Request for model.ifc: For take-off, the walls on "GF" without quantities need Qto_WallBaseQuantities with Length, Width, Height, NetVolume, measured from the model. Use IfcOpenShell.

First a look at what the model holds.

```python
import ifcopenshell
import ifcopenshell.util.element
import ifcopenshell.util.unit

model = ifcopenshell.open("model.ifc")
print(model.schema)
for unit_type in ("LENGTHUNIT", "AREAUNIT", "VOLUMEUNIT"):
    print(unit_type, ifcopenshell.util.unit.calculate_unit_scale(model, unit_type))
storey = next(s for s in model.by_type("IfcBuildingStorey") if s.Name == "GF")
walls = [e for e in ifcopenshell.util.element.get_decomposition(storey) if e.is_a("IfcWall")]
for e in sorted(walls, key=lambda e: e.id()):
    print(e.id(), e.is_a(), e.Name, list(ifcopenshell.util.element.get_psets(e, qtos_only=True)), sep=" | ")
```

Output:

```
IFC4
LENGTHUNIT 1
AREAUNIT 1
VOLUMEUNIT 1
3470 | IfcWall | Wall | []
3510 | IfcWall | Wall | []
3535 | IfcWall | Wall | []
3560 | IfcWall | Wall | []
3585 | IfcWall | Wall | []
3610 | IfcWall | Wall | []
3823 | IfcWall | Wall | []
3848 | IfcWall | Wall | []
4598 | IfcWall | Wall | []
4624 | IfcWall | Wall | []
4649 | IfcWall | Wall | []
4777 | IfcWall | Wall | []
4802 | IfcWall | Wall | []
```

```python
import ifcopenshell
import ifcopenshell.api.pset
import ifcopenshell.geom
import ifcopenshell.util.element
import ifcopenshell.util.shape
import ifcopenshell.util.unit

model = ifcopenshell.open("model.ifc")
unit_scale = ifcopenshell.util.unit.calculate_unit_scale(model)
volume_scale = ifcopenshell.util.unit.calculate_unit_scale(model, "VOLUMEUNIT")
settings = ifcopenshell.geom.settings()

storey = next(s for s in model.by_type("IfcBuildingStorey") if s.Name == "GF")
walls = [e for e in ifcopenshell.util.element.get_decomposition(storey) if e.is_a("IfcWall")]

for e in sorted(walls, key=lambda e: e.id()):
    if ifcopenshell.util.element.get_psets(e, qtos_only=True, should_inherit=False):
        continue
    # Geometry comes back in metres, in the element's own axes.
    shape = ifcopenshell.geom.create_shape(settings, e)
    values = {
        "Length": ifcopenshell.util.shape.get_x(shape.geometry) / unit_scale,
        "Width": ifcopenshell.util.shape.get_y(shape.geometry) / unit_scale,
        "Height": ifcopenshell.util.shape.get_z(shape.geometry) / unit_scale,
        "NetVolume": ifcopenshell.util.shape.get_volume(shape.geometry) / volume_scale,
    }
    qto = ifcopenshell.api.pset.add_qto(model, product=e, name="Qto_WallBaseQuantities")
    ifcopenshell.api.pset.edit_qto(model, qto=qto, properties=values)
    print(e.id(), {k: round(v, 3) for k, v in values.items()})

model.write("model_rev.ifc")
```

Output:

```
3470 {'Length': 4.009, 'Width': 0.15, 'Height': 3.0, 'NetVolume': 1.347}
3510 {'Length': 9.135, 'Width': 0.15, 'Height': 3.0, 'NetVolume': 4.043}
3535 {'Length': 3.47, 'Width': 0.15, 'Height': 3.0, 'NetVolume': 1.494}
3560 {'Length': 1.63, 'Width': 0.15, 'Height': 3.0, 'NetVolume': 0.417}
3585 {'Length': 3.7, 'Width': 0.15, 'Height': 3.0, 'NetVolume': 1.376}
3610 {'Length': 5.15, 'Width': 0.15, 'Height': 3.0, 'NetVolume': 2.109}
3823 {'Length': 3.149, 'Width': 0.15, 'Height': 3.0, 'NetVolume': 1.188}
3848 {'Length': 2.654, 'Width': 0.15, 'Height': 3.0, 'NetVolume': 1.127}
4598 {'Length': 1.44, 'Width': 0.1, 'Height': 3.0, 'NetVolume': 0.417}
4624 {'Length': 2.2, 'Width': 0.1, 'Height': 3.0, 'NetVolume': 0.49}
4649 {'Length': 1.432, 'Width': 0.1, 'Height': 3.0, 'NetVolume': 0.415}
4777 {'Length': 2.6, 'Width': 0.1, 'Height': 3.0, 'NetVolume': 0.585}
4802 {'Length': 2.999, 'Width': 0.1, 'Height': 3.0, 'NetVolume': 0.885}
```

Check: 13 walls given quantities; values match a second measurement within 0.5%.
